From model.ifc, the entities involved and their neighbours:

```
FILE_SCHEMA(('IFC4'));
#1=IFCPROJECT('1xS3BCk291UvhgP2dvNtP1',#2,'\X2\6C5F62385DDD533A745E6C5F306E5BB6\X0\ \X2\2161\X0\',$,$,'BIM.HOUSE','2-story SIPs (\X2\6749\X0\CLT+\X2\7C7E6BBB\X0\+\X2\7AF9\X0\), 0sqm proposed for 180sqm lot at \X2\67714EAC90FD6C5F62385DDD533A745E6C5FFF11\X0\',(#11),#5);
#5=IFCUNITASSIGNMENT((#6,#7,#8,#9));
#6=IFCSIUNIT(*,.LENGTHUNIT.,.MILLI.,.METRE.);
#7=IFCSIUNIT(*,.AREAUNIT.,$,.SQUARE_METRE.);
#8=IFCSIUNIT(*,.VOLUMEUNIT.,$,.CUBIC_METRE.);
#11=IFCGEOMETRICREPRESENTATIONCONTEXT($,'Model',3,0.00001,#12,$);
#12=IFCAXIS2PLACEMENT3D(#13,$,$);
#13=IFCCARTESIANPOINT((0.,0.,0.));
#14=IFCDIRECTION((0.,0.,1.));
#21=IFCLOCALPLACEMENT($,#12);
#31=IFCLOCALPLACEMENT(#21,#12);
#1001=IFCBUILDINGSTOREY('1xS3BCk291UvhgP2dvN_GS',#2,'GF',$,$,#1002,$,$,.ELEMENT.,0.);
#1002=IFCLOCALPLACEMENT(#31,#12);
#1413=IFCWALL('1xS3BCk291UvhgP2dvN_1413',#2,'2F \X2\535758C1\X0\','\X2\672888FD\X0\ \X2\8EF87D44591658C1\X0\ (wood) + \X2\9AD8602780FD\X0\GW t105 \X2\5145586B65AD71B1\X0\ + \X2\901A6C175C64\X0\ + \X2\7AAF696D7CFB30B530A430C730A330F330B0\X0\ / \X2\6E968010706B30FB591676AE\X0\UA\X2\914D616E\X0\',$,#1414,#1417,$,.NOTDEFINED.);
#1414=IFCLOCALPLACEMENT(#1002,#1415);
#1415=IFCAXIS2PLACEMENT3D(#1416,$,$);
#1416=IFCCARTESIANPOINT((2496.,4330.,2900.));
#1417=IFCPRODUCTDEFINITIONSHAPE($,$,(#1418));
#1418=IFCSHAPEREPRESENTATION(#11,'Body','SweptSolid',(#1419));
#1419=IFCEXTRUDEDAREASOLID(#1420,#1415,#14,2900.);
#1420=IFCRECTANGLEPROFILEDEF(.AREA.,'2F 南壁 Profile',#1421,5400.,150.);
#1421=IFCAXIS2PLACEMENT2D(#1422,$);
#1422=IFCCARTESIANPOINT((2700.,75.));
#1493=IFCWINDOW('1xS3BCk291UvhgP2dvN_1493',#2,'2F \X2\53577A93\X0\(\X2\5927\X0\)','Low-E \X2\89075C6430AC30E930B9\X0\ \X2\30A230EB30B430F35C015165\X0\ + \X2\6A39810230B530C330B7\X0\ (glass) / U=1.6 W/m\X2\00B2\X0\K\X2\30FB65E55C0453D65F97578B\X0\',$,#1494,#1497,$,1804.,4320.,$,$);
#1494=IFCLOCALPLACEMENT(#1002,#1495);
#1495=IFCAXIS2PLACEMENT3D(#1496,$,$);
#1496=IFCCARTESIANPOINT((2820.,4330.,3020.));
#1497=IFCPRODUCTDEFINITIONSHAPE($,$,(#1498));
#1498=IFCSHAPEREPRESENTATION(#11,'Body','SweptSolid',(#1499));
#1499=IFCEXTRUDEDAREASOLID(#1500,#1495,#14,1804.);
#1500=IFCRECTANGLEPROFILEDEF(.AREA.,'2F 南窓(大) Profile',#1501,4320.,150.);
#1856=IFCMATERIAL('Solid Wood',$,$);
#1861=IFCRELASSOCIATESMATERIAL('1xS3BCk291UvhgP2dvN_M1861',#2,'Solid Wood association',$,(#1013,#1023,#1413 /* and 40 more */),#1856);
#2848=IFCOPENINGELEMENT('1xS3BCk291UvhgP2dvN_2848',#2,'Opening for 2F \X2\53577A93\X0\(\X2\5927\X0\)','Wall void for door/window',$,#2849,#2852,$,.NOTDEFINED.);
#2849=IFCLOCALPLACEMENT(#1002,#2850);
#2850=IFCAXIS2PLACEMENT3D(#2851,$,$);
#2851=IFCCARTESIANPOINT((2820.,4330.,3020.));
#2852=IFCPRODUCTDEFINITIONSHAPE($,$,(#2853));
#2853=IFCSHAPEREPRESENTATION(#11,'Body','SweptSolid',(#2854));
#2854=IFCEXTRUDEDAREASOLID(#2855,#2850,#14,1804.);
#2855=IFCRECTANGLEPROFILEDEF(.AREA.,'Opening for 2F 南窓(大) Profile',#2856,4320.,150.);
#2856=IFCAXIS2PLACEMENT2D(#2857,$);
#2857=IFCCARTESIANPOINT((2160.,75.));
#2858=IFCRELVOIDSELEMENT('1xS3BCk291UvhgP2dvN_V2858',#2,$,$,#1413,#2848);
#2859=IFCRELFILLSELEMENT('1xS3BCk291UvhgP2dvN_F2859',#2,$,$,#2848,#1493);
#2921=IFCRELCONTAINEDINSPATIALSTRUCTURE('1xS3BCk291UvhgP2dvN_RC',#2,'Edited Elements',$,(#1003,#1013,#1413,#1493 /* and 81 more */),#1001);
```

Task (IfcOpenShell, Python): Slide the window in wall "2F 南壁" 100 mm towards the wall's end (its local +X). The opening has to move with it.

```python
import ifcopenshell
import ifcopenshell.api.geometry
import ifcopenshell.util.placement
import ifcopenshell.util.unit

model = ifcopenshell.open("model.ifc")
unit_scale = ifcopenshell.util.unit.calculate_unit_scale(model)

window = model.by_guid("1xS3BCk291UvhgP2dvN_1493")
opening = window.FillsVoids[0].RelatingOpeningElement
wall = opening.VoidsElements[0].RelatingBuildingElement

wall_matrix = ifcopenshell.util.placement.get_local_placement(wall.ObjectPlacement)
shift = wall_matrix[:3, 0] * 0.1 / unit_scale
before = ifcopenshell.util.placement.get_local_placement(window.ObjectPlacement)[:3, 3].copy()

# The window is not placed relative to its opening, so move both.
for product in (opening, window):
    matrix = ifcopenshell.util.placement.get_local_placement(product.ObjectPlacement)
    matrix[:3, 3] += shift
    ifcopenshell.api.geometry.edit_object_placement(model, product=product, matrix=matrix, is_si=False)

after = ifcopenshell.util.placement.get_local_placement(window.ObjectPlacement)[:3, 3]
print("window moved by", (after - before).round(3) + 0.0)

model.write("model_updated.ifc")
```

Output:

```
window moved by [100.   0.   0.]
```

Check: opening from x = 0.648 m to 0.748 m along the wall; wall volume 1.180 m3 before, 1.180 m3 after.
